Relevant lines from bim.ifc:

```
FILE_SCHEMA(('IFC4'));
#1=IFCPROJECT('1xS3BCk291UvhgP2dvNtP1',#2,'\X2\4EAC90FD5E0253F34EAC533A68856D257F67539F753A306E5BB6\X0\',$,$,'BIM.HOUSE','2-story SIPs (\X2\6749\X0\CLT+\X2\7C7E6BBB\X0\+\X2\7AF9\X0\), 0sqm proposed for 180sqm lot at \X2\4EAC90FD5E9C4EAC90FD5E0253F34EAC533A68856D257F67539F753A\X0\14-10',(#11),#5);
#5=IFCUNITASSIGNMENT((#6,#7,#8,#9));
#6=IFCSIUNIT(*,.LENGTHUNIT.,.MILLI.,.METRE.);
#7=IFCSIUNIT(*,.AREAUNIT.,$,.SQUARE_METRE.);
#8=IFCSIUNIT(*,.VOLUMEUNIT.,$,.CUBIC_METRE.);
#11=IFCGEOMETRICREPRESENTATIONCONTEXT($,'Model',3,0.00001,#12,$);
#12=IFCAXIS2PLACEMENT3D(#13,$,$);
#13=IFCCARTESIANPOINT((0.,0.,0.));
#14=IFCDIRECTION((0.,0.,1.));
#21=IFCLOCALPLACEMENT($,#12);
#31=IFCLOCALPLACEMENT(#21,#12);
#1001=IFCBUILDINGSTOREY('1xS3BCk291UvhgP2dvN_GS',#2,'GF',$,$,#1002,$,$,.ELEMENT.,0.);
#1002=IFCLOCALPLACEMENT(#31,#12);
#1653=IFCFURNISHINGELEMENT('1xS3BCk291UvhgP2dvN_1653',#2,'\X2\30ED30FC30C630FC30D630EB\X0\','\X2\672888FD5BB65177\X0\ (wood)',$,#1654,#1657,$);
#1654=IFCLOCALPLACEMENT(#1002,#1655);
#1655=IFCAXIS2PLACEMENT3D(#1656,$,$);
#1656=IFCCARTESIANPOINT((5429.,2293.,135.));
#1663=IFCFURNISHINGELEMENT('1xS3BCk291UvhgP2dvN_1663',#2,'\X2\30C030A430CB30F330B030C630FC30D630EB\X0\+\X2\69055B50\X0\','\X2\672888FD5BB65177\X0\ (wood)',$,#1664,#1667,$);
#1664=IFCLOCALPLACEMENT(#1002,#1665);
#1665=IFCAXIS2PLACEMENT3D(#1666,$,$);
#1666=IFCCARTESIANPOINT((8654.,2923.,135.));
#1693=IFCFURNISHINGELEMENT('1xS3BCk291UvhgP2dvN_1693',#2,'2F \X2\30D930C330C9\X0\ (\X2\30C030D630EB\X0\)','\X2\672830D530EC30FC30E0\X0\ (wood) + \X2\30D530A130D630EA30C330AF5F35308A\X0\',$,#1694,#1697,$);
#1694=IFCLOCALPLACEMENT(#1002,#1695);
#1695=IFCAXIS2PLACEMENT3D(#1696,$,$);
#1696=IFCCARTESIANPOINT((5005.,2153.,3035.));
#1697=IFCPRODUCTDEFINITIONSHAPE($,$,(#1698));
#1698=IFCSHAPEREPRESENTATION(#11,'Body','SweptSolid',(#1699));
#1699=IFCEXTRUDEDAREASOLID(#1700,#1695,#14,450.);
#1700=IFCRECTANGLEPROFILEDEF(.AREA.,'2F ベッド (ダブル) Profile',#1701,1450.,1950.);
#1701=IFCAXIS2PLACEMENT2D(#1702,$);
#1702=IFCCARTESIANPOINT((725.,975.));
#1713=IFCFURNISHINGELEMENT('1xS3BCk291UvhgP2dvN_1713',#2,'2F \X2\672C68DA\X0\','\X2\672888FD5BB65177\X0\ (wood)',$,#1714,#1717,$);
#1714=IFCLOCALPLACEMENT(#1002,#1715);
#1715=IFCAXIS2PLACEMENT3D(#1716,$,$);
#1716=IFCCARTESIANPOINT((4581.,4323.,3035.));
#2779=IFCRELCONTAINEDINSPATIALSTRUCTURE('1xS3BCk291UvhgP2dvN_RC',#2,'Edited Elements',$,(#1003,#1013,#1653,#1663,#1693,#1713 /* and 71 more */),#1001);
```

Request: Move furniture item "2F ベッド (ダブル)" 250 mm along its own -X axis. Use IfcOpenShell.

```python
import ifcopenshell
import ifcopenshell.api.geometry
import ifcopenshell.util.placement

model = ifcopenshell.open("bim.ifc")

item = model.by_guid("1xS3BCk291UvhgP2dvN_1693")
matrix = ifcopenshell.util.placement.get_local_placement(item.ObjectPlacement)
matrix[:3, 3] -= matrix[:3, 0] * 250.0
ifcopenshell.api.geometry.edit_object_placement(model, product=item, matrix=matrix, is_si=False)

print(ifcopenshell.util.placement.get_local_placement(item.ObjectPlacement).round(3) + 0.0)

model.write("bim_edited.ifc")
```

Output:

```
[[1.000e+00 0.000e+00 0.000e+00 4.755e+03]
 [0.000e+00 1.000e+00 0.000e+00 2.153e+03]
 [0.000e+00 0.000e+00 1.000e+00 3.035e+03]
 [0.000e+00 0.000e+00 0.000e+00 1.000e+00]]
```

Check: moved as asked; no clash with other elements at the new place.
